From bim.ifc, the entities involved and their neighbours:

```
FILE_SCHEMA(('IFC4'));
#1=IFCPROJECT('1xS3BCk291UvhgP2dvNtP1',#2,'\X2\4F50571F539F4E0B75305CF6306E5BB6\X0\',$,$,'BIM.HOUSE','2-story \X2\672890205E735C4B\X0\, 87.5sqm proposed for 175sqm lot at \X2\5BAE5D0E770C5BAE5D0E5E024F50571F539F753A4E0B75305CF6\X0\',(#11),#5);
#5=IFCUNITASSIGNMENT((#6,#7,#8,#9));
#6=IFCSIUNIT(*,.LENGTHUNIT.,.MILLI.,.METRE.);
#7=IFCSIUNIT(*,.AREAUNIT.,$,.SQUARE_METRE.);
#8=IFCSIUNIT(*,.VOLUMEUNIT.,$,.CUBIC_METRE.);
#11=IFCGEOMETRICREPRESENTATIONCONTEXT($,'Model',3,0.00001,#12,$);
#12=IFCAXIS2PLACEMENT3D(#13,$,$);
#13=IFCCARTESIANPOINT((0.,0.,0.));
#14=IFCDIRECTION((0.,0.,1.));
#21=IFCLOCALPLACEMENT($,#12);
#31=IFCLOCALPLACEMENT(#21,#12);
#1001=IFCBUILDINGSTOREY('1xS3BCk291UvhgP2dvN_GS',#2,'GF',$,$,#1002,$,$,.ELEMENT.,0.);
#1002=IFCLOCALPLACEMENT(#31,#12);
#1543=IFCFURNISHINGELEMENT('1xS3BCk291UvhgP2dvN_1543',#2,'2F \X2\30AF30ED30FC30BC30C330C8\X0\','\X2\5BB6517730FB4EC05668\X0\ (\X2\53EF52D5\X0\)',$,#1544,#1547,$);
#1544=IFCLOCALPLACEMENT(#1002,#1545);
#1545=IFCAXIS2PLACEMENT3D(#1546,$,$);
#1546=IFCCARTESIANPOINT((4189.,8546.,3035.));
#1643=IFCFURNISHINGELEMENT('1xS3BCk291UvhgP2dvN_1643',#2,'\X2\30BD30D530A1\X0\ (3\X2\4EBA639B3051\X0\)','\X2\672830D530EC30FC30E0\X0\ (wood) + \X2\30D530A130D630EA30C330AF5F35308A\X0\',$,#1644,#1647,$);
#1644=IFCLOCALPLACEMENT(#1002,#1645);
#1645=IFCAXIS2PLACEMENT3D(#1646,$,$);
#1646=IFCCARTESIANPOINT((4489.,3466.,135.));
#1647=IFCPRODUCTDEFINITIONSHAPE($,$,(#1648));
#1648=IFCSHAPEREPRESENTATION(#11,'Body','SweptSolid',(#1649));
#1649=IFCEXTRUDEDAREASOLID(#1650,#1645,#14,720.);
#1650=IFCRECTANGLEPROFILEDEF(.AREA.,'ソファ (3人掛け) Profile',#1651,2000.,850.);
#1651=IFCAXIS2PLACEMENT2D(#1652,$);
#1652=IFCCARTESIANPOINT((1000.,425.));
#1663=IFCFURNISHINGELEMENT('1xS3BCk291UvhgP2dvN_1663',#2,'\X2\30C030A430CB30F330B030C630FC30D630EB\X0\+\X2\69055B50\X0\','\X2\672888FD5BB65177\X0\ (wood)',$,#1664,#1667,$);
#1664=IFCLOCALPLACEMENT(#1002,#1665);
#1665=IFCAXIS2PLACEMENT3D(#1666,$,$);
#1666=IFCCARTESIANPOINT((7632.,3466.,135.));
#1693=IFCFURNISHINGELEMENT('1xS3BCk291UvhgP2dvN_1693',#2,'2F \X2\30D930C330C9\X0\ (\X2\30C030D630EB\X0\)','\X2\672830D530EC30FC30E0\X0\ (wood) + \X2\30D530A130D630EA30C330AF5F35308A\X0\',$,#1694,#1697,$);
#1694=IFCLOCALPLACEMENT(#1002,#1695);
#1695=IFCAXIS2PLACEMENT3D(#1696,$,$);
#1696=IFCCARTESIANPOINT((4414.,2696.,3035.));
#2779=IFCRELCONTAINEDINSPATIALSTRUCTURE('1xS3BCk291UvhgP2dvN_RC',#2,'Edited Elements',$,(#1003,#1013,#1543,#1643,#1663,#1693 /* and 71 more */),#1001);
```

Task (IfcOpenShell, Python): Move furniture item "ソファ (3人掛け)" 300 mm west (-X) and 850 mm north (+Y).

```python
import ifcopenshell
import ifcopenshell.api.geometry
import ifcopenshell.util.placement
import ifcopenshell.util.unit

model = ifcopenshell.open("bim.ifc")
unit_scale = ifcopenshell.util.unit.calculate_unit_scale(model)

item = model.by_id(1643)
matrix = ifcopenshell.util.placement.get_local_placement(item.ObjectPlacement)
matrix[0, 3] -= 0.3 / unit_scale
matrix[1, 3] += 0.85 / unit_scale
ifcopenshell.api.geometry.edit_object_placement(model, product=item, matrix=matrix, is_si=False)

print(ifcopenshell.util.placement.get_local_placement(item.ObjectPlacement).round(3) + 0.0)

model.write("bim_updated.ifc")
```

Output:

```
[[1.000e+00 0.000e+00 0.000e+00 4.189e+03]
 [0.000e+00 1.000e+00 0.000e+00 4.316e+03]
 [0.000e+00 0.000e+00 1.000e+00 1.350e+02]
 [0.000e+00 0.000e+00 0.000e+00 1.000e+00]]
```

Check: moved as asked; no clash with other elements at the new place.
